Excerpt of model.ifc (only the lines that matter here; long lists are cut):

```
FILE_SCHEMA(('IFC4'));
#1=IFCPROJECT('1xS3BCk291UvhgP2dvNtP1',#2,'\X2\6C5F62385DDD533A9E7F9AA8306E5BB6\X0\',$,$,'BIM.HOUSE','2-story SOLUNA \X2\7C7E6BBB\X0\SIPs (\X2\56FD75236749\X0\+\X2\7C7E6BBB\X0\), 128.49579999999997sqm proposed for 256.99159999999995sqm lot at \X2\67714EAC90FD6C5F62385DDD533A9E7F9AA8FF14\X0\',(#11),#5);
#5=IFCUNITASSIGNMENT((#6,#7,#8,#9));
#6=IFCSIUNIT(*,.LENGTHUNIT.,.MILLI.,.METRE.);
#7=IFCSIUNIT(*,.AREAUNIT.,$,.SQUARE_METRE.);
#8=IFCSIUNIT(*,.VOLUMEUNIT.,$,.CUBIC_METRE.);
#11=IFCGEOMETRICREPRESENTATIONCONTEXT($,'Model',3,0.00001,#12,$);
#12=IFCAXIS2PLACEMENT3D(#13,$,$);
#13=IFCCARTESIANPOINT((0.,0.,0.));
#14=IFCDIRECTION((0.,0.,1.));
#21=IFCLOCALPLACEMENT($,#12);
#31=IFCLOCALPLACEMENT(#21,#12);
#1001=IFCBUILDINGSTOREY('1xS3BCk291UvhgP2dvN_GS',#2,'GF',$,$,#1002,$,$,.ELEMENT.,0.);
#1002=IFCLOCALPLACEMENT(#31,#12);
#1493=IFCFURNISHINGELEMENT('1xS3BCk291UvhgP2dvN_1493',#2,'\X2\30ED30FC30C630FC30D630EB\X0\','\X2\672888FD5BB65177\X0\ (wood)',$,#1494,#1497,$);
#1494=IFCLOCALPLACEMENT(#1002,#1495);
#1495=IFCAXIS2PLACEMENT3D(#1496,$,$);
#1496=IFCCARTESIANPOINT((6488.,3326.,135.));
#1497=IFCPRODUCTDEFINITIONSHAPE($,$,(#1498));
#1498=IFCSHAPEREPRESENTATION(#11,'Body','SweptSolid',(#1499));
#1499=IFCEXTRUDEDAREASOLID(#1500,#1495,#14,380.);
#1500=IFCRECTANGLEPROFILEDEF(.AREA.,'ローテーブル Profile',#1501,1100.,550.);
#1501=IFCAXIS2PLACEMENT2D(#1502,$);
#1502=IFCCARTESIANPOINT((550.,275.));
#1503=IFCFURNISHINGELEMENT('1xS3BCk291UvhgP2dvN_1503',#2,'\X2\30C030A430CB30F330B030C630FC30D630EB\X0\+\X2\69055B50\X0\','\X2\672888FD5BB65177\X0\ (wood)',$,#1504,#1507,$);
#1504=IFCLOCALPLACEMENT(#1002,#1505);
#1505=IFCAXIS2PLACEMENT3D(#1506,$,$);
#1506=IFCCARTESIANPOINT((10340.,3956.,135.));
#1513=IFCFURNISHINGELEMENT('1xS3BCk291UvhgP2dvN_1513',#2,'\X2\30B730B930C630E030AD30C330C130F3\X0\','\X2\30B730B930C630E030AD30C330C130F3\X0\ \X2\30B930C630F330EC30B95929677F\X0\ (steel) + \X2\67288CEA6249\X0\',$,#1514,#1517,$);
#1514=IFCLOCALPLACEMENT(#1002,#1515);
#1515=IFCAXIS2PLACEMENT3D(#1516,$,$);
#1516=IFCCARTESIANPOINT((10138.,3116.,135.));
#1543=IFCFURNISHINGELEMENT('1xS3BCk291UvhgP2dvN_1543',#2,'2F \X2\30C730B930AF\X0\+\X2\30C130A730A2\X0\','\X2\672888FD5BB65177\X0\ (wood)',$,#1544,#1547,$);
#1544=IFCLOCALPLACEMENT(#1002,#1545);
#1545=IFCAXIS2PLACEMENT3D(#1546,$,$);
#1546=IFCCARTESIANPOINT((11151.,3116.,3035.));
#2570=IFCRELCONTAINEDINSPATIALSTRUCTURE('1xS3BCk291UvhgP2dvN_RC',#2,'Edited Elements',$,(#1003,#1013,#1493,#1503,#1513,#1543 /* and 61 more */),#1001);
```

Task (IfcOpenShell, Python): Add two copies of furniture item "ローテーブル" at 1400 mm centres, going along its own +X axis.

```python
import ifcopenshell
import ifcopenshell.api.geometry
import ifcopenshell.api.root
import ifcopenshell.util.element
import ifcopenshell.util.placement
import ifcopenshell.util.unit

model = ifcopenshell.open("model.ifc")
unit_scale = ifcopenshell.util.unit.calculate_unit_scale(model)


def reuse_history(source, copy):
    """copy_class also copies each property set's owner history, people and application; keep the originals."""
    for rel in copy.IsDefinedBy:
        if rel.is_a("IfcRelDefinesByProperties") and (history := rel.RelatingPropertyDefinition.OwnerHistory):
            rel.RelatingPropertyDefinition.OwnerHistory = source.OwnerHistory
            ifcopenshell.util.element.remove_deep2(model, history)


source = model.by_guid("1xS3BCk291UvhgP2dvN_1493")
base = ifcopenshell.util.placement.get_local_placement(source.ObjectPlacement)
step = base[:3, 0] * 1.4 / unit_scale

for i in range(1, 3):
    copy = ifcopenshell.api.root.copy_class(model, product=source)
    copy.Representation = ifcopenshell.util.element.copy_deep(
        model, source.Representation, exclude=["IfcGeometricRepresentationContext", "IfcRepresentationMap"]
    )
    reuse_history(source, copy)
    matrix = base.copy()
    matrix[:3, 3] += i * step
    print("added at", matrix[:3, 3].round(3) + 0.0)
    ifcopenshell.api.geometry.edit_object_placement(model, product=copy, matrix=matrix, is_si=False)

model.write("model_updated.ifc")
```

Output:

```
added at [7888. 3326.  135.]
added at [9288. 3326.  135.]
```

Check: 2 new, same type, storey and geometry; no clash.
